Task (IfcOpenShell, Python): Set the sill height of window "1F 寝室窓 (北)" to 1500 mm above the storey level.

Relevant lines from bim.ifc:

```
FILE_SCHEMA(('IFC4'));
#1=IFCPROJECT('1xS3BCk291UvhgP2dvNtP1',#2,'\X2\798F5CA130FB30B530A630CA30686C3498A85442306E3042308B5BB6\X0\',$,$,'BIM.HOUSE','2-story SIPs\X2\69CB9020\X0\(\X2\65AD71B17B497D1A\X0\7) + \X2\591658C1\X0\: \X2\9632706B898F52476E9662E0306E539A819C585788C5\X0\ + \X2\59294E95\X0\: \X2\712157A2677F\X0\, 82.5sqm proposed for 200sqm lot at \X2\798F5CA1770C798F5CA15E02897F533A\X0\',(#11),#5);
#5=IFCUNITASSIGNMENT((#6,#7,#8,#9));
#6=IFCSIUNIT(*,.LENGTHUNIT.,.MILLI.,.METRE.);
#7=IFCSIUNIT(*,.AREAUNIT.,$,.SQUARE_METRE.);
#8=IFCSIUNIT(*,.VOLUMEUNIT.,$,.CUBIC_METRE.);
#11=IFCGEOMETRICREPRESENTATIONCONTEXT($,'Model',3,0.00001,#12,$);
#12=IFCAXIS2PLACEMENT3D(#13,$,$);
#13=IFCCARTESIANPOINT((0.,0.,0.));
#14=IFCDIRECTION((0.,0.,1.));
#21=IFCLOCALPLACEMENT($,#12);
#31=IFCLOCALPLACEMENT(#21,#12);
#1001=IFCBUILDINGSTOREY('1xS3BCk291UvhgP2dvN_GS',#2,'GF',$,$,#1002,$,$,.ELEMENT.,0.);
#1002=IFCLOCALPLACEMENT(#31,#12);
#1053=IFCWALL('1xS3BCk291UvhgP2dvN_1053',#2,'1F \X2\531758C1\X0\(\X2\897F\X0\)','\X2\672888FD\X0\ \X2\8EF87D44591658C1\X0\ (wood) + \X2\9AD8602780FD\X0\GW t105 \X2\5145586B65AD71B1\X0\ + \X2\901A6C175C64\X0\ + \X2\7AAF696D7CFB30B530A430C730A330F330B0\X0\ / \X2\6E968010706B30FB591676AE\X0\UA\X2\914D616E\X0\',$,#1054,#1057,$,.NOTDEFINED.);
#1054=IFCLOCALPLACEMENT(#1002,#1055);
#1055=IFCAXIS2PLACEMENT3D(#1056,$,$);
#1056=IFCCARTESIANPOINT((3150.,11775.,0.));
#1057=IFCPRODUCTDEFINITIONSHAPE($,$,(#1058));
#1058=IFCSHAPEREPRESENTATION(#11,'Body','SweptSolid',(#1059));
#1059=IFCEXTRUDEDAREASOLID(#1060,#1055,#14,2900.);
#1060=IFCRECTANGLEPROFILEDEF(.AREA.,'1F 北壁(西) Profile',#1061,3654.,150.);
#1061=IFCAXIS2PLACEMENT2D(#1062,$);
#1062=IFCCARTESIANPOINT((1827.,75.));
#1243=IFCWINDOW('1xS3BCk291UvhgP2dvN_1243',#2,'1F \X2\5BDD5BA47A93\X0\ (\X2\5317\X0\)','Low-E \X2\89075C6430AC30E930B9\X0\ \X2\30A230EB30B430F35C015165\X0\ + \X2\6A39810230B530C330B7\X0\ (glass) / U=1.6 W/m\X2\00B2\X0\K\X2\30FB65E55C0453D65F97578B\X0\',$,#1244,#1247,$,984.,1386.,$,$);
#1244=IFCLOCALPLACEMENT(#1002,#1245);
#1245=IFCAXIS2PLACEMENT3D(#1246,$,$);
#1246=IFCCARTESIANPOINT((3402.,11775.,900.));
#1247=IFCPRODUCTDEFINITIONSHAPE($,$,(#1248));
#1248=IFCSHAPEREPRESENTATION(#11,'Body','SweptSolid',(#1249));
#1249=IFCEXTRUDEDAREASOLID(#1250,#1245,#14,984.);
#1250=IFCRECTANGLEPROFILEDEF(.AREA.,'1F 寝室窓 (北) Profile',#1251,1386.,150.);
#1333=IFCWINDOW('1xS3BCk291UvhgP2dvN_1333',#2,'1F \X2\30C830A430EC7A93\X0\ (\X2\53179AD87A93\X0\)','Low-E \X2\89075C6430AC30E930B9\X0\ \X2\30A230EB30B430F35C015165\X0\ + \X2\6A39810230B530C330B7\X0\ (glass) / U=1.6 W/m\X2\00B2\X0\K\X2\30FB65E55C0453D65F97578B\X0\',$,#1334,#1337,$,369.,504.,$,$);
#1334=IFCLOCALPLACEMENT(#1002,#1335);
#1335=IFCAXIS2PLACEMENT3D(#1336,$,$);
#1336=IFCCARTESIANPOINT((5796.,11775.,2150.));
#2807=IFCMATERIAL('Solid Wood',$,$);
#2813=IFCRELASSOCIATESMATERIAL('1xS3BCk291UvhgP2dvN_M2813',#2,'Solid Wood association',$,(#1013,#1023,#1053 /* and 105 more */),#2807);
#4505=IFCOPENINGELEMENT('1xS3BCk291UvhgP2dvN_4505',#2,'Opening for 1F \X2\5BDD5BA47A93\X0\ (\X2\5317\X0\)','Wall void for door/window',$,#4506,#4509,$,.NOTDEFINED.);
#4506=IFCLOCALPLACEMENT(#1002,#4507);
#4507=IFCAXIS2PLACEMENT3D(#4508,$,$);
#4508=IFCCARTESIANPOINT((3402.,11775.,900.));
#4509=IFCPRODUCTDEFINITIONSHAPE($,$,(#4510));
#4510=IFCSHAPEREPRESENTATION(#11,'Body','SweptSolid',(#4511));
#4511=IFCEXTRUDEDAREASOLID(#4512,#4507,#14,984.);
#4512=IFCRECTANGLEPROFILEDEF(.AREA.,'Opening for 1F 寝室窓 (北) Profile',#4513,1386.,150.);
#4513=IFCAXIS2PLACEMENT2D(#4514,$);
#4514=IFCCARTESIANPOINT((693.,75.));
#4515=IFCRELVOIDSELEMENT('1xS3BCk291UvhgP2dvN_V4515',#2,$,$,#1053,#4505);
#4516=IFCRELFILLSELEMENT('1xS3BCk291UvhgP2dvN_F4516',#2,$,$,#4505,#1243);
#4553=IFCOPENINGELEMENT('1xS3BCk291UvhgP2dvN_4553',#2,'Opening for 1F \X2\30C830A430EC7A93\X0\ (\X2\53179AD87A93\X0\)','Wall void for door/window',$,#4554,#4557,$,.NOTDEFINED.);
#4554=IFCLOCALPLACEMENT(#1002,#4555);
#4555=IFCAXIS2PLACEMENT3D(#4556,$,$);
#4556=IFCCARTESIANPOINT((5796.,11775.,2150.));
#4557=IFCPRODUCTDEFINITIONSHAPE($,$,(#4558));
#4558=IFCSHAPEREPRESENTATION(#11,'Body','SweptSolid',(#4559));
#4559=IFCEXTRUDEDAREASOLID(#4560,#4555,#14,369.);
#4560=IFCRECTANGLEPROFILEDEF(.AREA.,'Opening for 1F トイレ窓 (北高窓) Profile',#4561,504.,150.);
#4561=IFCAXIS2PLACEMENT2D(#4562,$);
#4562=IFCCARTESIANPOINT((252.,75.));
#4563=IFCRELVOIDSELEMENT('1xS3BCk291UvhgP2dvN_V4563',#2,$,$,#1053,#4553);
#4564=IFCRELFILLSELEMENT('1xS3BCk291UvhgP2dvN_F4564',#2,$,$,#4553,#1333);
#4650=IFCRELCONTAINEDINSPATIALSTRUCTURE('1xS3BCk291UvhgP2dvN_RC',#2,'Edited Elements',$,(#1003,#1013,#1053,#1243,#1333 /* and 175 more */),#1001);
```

```python
import numpy as np
import ifcopenshell
import ifcopenshell.api.geometry
import ifcopenshell.geom
import ifcopenshell.util.element
import ifcopenshell.util.placement
import ifcopenshell.util.shape
import ifcopenshell.util.unit

model = ifcopenshell.open("bim.ifc")
unit_scale = ifcopenshell.util.unit.calculate_unit_scale(model)

window = model.by_guid("1xS3BCk291UvhgP2dvN_1243")
opening = window.FillsVoids[0].RelatingOpeningElement
storey = ifcopenshell.util.element.get_container(window, ifc_class="IfcBuildingStorey")
level = ifcopenshell.util.placement.get_local_placement(storey.ObjectPlacement)[2, 3]

# The opening's origin need not be at the sill, so measure its lowest point.
shape = ifcopenshell.geom.create_shape(ifcopenshell.geom.settings(), opening)
bottom = ifcopenshell.util.shape.get_shape_bottom_elevation(shape, shape.geometry) / unit_scale
dz = level + 1.5 / unit_scale - bottom

shift = np.array([0.0, 0.0, dz])
# The window is not placed relative to its opening, so move both.
for product in (opening, window):
    matrix = ifcopenshell.util.placement.get_local_placement(product.ObjectPlacement)
    matrix[:3, 3] += shift
    ifcopenshell.api.geometry.edit_object_placement(model, product=product, matrix=matrix, is_si=False)

print(f"moved by {dz * unit_scale:+.3f} m")

model.write("bim_v2.ifc")
```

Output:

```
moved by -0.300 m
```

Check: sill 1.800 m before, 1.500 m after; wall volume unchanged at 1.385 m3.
